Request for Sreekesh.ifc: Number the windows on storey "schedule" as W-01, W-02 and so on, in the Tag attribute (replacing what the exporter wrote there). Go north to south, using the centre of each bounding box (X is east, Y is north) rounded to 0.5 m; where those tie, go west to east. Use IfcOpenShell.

First a look at what the model holds.

```python
import ifcopenshell
import ifcopenshell.util.element
import ifcopenshell.util.placement

model = ifcopenshell.open("Sreekesh.ifc")
print(model.schema)
storey = next(s for s in model.by_type("IfcBuildingStorey") if s.Name == "schedule")
windows = [e for e in ifcopenshell.util.element.get_decomposition(storey) if e.is_a("IfcWindow")]
for e in sorted(windows, key=lambda e: e.id()):
    origin = ifcopenshell.util.placement.get_local_placement(e.ObjectPlacement)[:3, 3]
    print(e.id(), e.Tag, e.Name, origin.round(2) + 0.0, sep=" | ")
```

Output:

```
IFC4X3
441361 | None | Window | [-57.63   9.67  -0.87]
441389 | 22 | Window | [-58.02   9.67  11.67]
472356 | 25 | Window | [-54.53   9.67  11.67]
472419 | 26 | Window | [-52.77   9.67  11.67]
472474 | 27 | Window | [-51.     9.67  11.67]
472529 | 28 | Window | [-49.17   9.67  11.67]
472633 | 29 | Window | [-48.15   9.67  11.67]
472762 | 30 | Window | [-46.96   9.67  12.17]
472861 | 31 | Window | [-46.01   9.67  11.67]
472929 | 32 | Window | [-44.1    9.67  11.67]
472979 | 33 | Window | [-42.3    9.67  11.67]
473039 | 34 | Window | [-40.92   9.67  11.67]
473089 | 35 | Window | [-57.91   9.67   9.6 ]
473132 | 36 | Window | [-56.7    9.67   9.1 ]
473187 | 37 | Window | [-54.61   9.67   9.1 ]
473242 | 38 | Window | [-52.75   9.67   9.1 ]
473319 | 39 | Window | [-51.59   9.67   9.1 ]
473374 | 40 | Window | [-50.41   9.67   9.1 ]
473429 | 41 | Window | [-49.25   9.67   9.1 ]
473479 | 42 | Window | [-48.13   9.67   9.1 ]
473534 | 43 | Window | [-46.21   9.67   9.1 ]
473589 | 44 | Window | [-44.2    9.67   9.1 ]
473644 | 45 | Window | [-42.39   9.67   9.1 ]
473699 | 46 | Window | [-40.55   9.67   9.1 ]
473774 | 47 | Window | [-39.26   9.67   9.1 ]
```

```python
import ifcopenshell
import ifcopenshell.geom
import ifcopenshell.util.element
import ifcopenshell.util.shape

model = ifcopenshell.open("Sreekesh.ifc")
settings = ifcopenshell.geom.settings()
settings.set("use-world-coords", True)


def centre(element):
    shape = ifcopenshell.geom.create_shape(settings, element)
    return ifcopenshell.util.shape.get_bbox_centroid(shape.geometry)


storey = next(s for s in model.by_type("IfcBuildingStorey") if s.Name == "schedule")
windows = [e for e in ifcopenshell.util.element.get_decomposition(storey) if e.is_a("IfcWindow")]

# Insertion points can sit at a corner or the storey origin, so sort by the geometry (in metres).
centres = {e: centre(e) for e in windows}
windows.sort(key=lambda e: (-round(centres[e][1] / 0.5), centres[e][0]))

for i, e in enumerate(windows, start=1):
    number = f"W-{i:02d}"
    e.Tag = number
    print(e.id(), number)

model.write("Sreekesh_updated.ifc")
```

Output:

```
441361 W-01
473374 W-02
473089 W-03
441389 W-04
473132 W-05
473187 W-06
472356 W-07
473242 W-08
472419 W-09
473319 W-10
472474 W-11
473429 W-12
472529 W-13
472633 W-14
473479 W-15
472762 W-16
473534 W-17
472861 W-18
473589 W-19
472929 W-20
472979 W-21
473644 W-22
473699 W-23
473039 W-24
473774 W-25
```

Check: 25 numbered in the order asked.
